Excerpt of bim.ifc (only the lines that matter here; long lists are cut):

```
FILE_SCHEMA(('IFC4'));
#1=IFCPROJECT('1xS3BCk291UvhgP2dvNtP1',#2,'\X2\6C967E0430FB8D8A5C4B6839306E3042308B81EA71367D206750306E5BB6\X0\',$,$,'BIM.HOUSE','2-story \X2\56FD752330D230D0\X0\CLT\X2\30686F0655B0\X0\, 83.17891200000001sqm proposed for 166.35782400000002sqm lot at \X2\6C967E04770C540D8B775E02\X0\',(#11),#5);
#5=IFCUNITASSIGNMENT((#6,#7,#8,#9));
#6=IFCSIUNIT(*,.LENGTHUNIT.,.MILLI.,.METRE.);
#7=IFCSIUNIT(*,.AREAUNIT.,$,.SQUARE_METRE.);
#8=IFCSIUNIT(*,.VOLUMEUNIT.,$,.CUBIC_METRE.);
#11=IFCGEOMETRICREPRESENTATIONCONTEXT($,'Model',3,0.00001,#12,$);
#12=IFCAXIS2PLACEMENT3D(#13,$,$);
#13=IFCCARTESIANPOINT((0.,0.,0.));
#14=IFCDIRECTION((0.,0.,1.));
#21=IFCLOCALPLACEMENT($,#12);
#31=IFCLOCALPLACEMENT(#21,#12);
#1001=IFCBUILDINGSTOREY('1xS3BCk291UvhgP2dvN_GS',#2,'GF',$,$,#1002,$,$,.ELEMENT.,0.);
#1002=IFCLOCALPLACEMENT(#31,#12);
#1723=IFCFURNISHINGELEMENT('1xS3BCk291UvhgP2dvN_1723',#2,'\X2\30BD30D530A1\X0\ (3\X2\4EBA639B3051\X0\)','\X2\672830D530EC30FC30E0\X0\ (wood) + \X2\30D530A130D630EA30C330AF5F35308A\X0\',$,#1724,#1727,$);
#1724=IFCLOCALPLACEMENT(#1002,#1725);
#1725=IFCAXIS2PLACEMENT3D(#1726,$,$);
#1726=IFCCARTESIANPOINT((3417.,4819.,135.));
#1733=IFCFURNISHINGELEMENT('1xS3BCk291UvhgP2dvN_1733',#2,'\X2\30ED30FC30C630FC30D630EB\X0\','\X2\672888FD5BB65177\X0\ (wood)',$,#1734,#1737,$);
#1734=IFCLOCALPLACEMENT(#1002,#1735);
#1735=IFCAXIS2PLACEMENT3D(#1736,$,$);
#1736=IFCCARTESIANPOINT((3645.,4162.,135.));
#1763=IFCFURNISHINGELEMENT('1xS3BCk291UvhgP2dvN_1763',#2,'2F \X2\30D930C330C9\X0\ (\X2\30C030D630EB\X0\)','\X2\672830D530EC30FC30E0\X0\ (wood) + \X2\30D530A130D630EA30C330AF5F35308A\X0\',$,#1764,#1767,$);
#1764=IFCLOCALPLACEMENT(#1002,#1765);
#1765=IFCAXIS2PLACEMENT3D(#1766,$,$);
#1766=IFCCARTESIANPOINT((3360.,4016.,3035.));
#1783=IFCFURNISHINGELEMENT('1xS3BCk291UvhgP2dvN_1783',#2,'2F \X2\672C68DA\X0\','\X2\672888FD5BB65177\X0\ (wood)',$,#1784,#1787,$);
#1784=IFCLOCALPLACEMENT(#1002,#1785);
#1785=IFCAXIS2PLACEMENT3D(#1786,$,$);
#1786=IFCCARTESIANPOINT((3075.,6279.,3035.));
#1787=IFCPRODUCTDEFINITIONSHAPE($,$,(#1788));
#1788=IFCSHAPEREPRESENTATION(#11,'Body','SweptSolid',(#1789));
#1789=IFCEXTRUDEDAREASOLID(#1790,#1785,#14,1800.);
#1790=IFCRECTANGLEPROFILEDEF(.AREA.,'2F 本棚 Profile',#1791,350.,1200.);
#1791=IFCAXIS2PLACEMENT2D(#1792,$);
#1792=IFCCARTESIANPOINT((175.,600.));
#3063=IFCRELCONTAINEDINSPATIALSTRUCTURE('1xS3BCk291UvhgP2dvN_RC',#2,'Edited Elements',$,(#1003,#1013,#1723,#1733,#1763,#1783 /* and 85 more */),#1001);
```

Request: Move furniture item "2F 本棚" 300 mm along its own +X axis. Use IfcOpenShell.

```python
import ifcopenshell
import ifcopenshell.api.geometry
import ifcopenshell.util.placement

model = ifcopenshell.open("bim.ifc")

item = model.by_guid("1xS3BCk291UvhgP2dvN_1783")
matrix = ifcopenshell.util.placement.get_local_placement(item.ObjectPlacement)
matrix[:3, 3] += matrix[:3, 0] * 300.0
ifcopenshell.api.geometry.edit_object_placement(model, product=item, matrix=matrix, is_si=False)

print(ifcopenshell.util.placement.get_local_placement(item.ObjectPlacement).round(3) + 0.0)

model.write("bim_rev.ifc")
```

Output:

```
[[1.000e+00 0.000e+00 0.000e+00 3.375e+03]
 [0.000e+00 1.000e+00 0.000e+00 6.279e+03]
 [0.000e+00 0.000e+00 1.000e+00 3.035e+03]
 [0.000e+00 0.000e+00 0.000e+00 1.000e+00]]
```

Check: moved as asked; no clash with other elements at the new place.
